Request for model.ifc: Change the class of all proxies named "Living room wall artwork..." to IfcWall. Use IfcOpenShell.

First a look at what the model holds.

```python
import re

import ifcopenshell

model = ifcopenshell.open("model.ifc")
print(model.schema)
seen = {}
for e in model.by_type("IfcBuildingElementProxy"):
    name = re.sub(r":\d+(:\d+)?$", "", e.Name or "")  # drop the element id that some exporters append
    seen[name] = seen.get(name, 0) + 1
for name, count in sorted(seen.items()):
    print(count, "x", name)
```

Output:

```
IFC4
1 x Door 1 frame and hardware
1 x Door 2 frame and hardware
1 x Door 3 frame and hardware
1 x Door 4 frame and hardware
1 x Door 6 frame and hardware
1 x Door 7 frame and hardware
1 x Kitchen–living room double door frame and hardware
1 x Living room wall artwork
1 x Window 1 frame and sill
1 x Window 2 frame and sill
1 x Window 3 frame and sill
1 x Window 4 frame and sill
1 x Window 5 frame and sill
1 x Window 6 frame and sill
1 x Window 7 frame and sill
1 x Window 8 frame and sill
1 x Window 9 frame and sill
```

```python
import ifcopenshell
import ifcopenshell.api.root

model = ifcopenshell.open("model.ifc")

proxies = [e.id() for e in model.by_type("IfcBuildingElementProxy") if (e.Name or "").startswith("Living room wall artwork")]
for step_id in proxies:
    proxy = model.by_id(step_id)
    ifcopenshell.api.root.reassign_class(model, product=proxy, ifc_class="IfcWall")

print(sum(model.by_id(i).is_a("IfcWall") for i in proxies), "reclassified")

model.write("model_updated.ifc")
```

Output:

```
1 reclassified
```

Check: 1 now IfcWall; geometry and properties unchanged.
